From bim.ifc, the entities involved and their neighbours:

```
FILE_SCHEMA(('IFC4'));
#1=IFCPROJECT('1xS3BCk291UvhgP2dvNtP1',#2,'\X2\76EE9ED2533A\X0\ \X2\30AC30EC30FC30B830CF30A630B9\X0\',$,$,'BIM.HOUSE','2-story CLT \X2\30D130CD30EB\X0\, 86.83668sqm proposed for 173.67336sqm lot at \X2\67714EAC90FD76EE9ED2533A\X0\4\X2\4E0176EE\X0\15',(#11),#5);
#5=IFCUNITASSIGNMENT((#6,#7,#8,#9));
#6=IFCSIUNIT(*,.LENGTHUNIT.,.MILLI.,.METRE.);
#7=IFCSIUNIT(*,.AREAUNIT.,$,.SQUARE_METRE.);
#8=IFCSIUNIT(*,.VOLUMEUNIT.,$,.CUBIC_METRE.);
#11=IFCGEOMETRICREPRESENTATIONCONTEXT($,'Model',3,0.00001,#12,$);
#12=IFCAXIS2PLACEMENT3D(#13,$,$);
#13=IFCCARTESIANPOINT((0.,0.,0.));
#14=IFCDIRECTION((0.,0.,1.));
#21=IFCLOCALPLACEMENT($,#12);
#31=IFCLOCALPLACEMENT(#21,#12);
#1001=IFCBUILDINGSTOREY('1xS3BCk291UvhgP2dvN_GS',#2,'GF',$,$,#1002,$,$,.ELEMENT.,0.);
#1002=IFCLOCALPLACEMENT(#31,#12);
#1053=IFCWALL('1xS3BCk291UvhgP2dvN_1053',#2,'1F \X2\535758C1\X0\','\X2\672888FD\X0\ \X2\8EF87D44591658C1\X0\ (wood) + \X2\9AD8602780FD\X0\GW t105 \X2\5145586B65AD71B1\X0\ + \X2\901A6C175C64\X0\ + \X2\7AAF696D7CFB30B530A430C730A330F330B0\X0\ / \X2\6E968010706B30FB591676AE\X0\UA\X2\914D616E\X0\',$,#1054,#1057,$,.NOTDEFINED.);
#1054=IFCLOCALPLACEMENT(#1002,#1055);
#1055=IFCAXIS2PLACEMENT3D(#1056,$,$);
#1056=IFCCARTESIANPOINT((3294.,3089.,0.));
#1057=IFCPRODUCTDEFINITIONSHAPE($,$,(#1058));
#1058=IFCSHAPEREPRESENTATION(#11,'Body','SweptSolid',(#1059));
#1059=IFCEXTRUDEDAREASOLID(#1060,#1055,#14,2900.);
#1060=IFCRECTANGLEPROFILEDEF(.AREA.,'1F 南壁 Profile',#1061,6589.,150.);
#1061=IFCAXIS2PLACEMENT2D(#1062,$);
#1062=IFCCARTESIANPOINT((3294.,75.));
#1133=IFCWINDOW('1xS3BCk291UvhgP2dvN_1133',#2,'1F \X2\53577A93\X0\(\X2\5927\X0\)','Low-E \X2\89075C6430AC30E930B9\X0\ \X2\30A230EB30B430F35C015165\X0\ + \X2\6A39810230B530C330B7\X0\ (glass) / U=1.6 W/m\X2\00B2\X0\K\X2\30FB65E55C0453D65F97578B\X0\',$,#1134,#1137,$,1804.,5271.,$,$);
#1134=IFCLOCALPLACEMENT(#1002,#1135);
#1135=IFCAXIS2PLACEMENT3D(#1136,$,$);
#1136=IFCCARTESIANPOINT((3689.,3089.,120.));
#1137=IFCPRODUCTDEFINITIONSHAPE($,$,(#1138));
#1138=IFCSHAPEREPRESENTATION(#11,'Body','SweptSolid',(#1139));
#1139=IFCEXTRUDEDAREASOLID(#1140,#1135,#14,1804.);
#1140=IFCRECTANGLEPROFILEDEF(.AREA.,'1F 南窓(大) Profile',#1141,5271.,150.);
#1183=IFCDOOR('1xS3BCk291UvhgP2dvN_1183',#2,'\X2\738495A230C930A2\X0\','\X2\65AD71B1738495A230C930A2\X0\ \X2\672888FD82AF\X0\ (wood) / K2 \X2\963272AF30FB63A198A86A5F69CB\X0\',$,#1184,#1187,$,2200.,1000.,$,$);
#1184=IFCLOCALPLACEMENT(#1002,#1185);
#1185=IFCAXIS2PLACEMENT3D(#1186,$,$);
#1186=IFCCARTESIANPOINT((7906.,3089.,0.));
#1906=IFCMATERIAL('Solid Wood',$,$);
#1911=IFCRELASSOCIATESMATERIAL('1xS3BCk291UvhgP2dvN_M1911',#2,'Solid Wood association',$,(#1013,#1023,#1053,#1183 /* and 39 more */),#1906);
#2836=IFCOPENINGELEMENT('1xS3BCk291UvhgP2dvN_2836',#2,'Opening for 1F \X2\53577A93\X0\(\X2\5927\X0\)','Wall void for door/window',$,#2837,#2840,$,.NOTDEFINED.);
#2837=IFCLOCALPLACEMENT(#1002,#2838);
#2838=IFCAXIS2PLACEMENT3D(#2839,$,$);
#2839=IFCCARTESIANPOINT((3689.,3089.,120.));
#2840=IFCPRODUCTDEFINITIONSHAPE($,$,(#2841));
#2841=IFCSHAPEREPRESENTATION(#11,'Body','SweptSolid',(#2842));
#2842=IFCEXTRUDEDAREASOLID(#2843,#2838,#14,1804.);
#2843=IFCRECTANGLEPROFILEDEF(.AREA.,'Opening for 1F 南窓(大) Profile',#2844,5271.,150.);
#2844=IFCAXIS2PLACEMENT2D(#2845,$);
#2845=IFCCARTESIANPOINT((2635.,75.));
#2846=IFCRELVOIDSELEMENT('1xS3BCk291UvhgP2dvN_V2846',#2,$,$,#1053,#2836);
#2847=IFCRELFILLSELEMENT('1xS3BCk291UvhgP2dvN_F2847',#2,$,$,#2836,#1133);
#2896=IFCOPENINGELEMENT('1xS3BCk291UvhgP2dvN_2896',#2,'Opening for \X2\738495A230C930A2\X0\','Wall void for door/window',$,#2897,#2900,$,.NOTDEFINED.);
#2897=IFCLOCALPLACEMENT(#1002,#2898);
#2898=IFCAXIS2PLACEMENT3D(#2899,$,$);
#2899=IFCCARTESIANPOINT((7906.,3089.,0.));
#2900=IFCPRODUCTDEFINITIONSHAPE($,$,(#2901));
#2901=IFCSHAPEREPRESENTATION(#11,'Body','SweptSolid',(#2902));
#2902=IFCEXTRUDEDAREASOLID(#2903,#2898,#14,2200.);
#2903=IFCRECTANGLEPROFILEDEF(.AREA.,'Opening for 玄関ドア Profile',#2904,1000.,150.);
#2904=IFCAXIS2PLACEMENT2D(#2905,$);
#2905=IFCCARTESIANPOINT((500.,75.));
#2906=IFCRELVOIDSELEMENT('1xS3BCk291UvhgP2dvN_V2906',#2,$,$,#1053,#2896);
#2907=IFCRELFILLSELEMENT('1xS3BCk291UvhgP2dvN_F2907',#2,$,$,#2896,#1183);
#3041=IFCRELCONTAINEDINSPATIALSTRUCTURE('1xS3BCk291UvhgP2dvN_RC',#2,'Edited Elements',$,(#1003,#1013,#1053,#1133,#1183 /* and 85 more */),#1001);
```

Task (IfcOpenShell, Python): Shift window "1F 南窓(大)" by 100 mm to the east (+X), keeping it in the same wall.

```python
import ifcopenshell
import ifcopenshell.api.geometry
import ifcopenshell.util.placement
import ifcopenshell.util.unit

model = ifcopenshell.open("bim.ifc")
unit_scale = ifcopenshell.util.unit.calculate_unit_scale(model)

window = model.by_id(1133)
opening = window.FillsVoids[0].RelatingOpeningElement
wall = opening.VoidsElements[0].RelatingBuildingElement

wall_matrix = ifcopenshell.util.placement.get_local_placement(wall.ObjectPlacement)
shift = wall_matrix[:3, 0] * 0.1 / unit_scale
before = ifcopenshell.util.placement.get_local_placement(window.ObjectPlacement)[:3, 3].copy()

# The window is not placed relative to its opening, so move both.
for product in (opening, window):
    matrix = ifcopenshell.util.placement.get_local_placement(product.ObjectPlacement)
    matrix[:3, 3] += shift
    ifcopenshell.api.geometry.edit_object_placement(model, product=product, matrix=matrix, is_si=False)

after = ifcopenshell.util.placement.get_local_placement(window.ObjectPlacement)[:3, 3]
print("window moved by", (after - before).round(3) + 0.0)

model.write("bim-out.ifc")
```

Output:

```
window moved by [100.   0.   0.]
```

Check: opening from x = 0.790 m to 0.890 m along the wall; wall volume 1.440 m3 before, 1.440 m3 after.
